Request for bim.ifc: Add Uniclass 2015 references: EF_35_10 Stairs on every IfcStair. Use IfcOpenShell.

First a look at what the model holds.

```python
import ifcopenshell

model = ifcopenshell.open("bim.ifc")
print(model.schema)
print("classifications:", [c.Name for c in model.by_type("IfcClassification")])
for ifc_class in ("IfcDoor", "IfcRoof", "IfcStair", "IfcWall", "IfcWindow"):
    print(ifc_class, len(model.by_type(ifc_class)))
```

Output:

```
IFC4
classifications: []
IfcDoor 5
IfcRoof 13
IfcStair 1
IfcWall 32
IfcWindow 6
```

```python
import ifcopenshell
import ifcopenshell.api.classification

model = ifcopenshell.open("bim.ifc")

system = ifcopenshell.api.classification.add_classification(model, classification="Uniclass 2015")

codes = {
    "IfcStair": ("EF_35_10", "Stairs"),
}
for ifc_class, (code, name) in codes.items():
    products = model.by_type(ifc_class)
    ifcopenshell.api.classification.add_reference(
        model, products=products, classification=system, identification=code, name=name
    )
    print(code, len(products))

model.write("bim_edited.ifc")
```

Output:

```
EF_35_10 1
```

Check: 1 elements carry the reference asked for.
